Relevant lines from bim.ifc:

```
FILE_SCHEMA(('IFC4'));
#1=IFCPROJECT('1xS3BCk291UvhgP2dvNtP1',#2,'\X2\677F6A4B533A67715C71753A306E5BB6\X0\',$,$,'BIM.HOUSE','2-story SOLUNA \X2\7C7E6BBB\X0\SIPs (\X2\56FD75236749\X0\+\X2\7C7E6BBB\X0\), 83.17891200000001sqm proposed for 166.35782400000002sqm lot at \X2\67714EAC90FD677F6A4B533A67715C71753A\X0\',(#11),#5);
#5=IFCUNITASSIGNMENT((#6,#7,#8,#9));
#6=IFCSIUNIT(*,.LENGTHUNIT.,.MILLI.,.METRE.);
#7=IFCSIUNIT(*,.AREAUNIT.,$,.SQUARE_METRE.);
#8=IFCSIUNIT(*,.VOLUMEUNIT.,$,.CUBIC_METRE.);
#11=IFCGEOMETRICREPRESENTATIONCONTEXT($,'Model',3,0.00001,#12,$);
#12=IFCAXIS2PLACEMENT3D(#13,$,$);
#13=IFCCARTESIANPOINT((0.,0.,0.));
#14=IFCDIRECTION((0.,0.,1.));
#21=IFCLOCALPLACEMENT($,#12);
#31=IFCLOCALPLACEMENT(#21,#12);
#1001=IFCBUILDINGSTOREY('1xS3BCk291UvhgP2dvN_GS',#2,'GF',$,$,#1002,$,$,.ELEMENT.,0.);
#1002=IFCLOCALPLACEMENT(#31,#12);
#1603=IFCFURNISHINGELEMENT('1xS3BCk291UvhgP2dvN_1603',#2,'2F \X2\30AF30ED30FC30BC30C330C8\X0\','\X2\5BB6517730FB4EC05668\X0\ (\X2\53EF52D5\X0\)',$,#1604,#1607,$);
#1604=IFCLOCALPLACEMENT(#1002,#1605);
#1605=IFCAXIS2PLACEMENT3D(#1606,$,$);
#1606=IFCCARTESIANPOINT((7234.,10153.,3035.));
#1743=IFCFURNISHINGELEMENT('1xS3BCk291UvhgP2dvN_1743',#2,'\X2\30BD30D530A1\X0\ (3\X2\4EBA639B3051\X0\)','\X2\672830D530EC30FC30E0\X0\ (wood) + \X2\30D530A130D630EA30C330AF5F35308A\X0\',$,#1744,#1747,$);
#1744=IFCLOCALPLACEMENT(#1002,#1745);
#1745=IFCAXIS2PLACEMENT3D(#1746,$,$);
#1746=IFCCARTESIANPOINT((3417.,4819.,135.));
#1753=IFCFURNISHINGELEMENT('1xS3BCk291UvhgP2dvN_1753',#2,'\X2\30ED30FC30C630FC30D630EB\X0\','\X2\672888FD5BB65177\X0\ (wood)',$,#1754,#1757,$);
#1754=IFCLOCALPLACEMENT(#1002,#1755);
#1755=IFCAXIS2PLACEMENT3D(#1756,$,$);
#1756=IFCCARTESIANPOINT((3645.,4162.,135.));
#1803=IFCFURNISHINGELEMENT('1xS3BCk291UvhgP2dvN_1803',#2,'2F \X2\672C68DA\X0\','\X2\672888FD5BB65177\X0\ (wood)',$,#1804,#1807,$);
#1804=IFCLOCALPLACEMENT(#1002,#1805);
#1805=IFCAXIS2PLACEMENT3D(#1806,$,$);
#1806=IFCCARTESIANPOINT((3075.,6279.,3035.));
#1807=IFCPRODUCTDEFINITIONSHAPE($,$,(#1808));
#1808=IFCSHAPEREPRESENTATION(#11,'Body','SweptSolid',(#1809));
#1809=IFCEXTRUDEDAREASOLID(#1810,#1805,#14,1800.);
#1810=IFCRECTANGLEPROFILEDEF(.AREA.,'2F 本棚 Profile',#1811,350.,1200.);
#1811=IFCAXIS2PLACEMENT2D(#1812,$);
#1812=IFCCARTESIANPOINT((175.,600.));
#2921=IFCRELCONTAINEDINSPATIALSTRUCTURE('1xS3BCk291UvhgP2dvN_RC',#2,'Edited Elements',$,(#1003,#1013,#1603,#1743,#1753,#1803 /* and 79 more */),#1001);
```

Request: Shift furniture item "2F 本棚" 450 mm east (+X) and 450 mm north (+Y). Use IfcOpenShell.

```python
import ifcopenshell
import ifcopenshell.api.geometry
import ifcopenshell.util.placement
import ifcopenshell.util.unit

model = ifcopenshell.open("bim.ifc")
unit_scale = ifcopenshell.util.unit.calculate_unit_scale(model)

item = model.by_guid("1xS3BCk291UvhgP2dvN_1803")
matrix = ifcopenshell.util.placement.get_local_placement(item.ObjectPlacement)
matrix[0, 3] += 0.45 / unit_scale
matrix[1, 3] += 0.45 / unit_scale
ifcopenshell.api.geometry.edit_object_placement(model, product=item, matrix=matrix, is_si=False)

print(ifcopenshell.util.placement.get_local_placement(item.ObjectPlacement).round(3) + 0.0)

model.write("bim_edited.ifc")
```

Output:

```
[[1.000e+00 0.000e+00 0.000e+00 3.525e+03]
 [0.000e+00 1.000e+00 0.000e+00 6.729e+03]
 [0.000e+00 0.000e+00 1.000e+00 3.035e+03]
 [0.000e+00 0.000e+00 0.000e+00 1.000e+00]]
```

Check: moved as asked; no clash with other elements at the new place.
